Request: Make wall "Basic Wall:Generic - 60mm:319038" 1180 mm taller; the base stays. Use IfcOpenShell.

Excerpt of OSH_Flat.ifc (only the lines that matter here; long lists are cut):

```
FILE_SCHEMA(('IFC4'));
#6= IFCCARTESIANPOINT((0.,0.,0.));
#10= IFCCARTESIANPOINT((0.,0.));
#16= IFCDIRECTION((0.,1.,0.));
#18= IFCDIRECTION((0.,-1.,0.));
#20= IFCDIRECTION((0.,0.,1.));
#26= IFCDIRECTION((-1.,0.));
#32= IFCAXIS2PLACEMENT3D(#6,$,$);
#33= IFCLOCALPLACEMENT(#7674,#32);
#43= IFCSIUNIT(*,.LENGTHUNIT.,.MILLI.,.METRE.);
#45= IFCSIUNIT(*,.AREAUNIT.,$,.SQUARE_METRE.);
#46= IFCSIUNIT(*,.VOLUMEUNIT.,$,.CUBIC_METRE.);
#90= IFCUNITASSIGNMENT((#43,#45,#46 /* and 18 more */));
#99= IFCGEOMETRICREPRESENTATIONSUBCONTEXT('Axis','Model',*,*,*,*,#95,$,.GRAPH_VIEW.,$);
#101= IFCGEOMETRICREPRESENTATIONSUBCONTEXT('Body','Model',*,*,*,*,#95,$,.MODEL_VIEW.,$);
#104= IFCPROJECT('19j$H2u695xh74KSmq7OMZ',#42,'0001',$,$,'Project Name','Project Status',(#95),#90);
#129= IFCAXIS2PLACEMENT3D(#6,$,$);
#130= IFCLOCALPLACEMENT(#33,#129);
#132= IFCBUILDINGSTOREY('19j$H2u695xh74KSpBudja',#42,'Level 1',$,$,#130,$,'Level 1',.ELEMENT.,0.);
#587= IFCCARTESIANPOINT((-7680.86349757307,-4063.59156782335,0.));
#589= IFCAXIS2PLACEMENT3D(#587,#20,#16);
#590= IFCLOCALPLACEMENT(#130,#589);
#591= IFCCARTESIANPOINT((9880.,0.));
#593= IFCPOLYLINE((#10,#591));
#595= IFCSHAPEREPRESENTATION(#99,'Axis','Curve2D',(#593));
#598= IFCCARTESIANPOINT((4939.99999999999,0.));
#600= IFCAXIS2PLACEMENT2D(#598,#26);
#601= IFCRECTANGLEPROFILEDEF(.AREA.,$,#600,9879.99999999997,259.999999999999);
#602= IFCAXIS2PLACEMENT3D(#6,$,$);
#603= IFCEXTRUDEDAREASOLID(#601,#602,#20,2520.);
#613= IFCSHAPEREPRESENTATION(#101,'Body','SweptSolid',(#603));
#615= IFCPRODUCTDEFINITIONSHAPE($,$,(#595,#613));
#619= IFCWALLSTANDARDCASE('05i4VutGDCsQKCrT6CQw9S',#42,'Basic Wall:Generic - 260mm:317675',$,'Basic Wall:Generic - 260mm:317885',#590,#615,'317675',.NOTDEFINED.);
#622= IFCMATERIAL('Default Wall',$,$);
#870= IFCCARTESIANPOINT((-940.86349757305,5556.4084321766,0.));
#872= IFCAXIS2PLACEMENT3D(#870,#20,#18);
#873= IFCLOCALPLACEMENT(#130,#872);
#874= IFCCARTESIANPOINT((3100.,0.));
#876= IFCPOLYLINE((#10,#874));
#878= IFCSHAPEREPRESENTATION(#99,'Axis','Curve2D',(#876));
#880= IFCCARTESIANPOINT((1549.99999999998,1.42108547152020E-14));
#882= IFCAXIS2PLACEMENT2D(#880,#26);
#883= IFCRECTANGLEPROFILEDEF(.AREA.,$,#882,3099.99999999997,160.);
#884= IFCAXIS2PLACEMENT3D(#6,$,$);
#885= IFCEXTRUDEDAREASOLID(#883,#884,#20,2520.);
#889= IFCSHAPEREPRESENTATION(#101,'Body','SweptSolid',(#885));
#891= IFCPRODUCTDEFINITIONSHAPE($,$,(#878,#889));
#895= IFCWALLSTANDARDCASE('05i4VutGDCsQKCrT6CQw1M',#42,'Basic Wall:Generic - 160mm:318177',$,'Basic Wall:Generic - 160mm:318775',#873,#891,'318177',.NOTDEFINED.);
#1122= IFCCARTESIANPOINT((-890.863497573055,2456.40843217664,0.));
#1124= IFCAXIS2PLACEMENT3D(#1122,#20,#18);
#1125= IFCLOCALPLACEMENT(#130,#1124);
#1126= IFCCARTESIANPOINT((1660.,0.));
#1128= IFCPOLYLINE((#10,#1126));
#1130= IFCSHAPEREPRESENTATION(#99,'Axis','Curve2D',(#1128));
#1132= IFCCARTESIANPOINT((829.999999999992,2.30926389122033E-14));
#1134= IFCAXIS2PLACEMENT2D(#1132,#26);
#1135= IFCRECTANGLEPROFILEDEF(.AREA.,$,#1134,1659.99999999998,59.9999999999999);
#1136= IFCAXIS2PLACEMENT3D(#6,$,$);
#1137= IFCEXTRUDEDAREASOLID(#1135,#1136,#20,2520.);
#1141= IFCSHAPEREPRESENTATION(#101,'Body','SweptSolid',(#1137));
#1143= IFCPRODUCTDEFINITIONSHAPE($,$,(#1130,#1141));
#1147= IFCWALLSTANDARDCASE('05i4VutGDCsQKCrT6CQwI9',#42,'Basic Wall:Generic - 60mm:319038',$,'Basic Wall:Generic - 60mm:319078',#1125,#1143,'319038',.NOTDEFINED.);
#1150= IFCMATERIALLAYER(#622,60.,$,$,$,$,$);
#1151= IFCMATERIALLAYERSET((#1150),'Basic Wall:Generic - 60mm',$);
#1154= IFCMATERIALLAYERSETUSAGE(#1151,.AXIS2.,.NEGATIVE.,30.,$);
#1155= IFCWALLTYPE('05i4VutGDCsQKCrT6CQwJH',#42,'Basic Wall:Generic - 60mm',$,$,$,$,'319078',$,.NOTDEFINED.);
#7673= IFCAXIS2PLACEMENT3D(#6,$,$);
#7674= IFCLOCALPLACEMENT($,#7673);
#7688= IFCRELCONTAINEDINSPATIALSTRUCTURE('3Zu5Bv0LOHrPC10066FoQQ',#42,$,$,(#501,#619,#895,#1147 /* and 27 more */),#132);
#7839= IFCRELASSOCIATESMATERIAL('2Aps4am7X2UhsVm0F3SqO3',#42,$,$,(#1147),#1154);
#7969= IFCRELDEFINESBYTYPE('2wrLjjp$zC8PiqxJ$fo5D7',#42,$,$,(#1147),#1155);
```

```python
import ifcopenshell
import ifcopenshell.geom
import ifcopenshell.util.representation
import ifcopenshell.util.shape
import ifcopenshell.util.unit

model = ifcopenshell.open("OSH_Flat.ifc")
unit_scale = ifcopenshell.util.unit.calculate_unit_scale(model)
settings = ifcopenshell.geom.settings()


def volume(element):
    """Net volume in cubic metres, openings subtracted."""
    shape = ifcopenshell.geom.create_shape(settings, element)
    return ifcopenshell.util.shape.get_volume(shape.geometry)


wall = model.by_id(1147)
before = volume(wall)

body = ifcopenshell.util.representation.get_representation(wall, "Model", "Body")
solid = body.Items[0]
old_height = solid.Depth
solid.Depth += 1.18 / unit_scale
after = volume(wall)

print(f"height {old_height:g} -> {solid.Depth:g}, volume {before:.3f} -> {after:.3f} m3")

model.write("OSH_Flat_updated.ifc")
```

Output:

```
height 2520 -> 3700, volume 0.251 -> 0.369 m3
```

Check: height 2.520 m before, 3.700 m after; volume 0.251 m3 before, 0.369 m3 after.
